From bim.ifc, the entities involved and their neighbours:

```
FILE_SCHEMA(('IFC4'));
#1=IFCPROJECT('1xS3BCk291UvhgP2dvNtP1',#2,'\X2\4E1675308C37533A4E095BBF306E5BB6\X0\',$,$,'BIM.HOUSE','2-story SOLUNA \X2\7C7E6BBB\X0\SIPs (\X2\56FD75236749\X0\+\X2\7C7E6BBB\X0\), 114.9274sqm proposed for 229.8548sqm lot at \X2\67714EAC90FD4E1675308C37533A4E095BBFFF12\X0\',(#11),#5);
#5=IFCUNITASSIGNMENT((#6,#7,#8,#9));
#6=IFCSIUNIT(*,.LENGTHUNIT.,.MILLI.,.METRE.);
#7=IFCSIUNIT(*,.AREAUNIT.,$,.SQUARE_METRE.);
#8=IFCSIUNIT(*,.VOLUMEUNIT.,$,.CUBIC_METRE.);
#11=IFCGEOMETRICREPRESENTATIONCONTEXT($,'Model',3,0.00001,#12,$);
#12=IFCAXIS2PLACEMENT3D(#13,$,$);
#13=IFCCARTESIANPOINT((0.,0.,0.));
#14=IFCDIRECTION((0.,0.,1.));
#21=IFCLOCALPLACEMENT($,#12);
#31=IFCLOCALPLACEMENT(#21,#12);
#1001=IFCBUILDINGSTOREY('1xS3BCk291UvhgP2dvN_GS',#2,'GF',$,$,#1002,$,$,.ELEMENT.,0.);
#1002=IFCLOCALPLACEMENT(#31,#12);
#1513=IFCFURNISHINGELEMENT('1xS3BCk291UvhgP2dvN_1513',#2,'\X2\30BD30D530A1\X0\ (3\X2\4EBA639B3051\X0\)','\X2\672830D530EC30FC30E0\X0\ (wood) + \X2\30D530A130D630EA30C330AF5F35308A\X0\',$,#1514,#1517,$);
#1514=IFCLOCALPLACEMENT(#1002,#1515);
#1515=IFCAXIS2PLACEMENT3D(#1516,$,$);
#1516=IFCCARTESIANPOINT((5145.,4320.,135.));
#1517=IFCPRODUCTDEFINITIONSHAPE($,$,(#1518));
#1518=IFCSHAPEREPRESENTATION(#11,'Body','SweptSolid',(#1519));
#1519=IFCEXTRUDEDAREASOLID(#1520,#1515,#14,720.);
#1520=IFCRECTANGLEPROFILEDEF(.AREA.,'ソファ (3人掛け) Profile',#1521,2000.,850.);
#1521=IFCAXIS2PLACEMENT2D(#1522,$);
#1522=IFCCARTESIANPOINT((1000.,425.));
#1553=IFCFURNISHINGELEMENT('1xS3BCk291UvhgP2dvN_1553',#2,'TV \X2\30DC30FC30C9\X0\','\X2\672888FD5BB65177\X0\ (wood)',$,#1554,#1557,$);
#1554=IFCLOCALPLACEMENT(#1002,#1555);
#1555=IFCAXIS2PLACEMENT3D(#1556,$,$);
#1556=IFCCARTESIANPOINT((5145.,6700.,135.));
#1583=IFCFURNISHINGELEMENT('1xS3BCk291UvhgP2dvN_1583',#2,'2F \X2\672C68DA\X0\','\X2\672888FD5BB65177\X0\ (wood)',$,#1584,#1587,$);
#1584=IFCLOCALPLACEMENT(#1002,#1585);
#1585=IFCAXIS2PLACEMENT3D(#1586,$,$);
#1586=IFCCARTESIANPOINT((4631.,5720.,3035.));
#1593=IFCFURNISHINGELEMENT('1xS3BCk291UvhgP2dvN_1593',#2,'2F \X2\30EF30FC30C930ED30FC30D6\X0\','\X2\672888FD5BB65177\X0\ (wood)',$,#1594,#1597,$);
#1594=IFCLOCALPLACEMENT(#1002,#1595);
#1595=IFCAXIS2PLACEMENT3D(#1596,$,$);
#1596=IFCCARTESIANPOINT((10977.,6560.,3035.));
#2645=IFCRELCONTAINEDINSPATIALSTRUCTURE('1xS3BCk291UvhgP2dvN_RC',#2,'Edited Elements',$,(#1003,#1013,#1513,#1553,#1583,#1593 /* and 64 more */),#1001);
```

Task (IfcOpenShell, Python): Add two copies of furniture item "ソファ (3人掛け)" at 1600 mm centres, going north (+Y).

```python
import numpy as np
import ifcopenshell
import ifcopenshell.api.geometry
import ifcopenshell.api.root
import ifcopenshell.util.element
import ifcopenshell.util.placement
import ifcopenshell.util.unit

model = ifcopenshell.open("bim.ifc")
unit_scale = ifcopenshell.util.unit.calculate_unit_scale(model)


def reuse_history(source, copy):
    """copy_class also copies each property set's owner history, people and application; keep the originals."""
    for rel in copy.IsDefinedBy:
        if rel.is_a("IfcRelDefinesByProperties") and (history := rel.RelatingPropertyDefinition.OwnerHistory):
            rel.RelatingPropertyDefinition.OwnerHistory = source.OwnerHistory
            ifcopenshell.util.element.remove_deep2(model, history)


source = model.by_guid("1xS3BCk291UvhgP2dvN_1513")
base = ifcopenshell.util.placement.get_local_placement(source.ObjectPlacement)
step = np.array([0.0, 1.0, 0.0]) * 1.6 / unit_scale

for i in range(1, 3):
    copy = ifcopenshell.api.root.copy_class(model, product=source)
    copy.Representation = ifcopenshell.util.element.copy_deep(
        model, source.Representation, exclude=["IfcGeometricRepresentationContext", "IfcRepresentationMap"]
    )
    reuse_history(source, copy)
    matrix = base.copy()
    matrix[:3, 3] += i * step
    print("added at", matrix[:3, 3].round(3) + 0.0)
    ifcopenshell.api.geometry.edit_object_placement(model, product=copy, matrix=matrix, is_si=False)

model.write("bim_v2.ifc")
```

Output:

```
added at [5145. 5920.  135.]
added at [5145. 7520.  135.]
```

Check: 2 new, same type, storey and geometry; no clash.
